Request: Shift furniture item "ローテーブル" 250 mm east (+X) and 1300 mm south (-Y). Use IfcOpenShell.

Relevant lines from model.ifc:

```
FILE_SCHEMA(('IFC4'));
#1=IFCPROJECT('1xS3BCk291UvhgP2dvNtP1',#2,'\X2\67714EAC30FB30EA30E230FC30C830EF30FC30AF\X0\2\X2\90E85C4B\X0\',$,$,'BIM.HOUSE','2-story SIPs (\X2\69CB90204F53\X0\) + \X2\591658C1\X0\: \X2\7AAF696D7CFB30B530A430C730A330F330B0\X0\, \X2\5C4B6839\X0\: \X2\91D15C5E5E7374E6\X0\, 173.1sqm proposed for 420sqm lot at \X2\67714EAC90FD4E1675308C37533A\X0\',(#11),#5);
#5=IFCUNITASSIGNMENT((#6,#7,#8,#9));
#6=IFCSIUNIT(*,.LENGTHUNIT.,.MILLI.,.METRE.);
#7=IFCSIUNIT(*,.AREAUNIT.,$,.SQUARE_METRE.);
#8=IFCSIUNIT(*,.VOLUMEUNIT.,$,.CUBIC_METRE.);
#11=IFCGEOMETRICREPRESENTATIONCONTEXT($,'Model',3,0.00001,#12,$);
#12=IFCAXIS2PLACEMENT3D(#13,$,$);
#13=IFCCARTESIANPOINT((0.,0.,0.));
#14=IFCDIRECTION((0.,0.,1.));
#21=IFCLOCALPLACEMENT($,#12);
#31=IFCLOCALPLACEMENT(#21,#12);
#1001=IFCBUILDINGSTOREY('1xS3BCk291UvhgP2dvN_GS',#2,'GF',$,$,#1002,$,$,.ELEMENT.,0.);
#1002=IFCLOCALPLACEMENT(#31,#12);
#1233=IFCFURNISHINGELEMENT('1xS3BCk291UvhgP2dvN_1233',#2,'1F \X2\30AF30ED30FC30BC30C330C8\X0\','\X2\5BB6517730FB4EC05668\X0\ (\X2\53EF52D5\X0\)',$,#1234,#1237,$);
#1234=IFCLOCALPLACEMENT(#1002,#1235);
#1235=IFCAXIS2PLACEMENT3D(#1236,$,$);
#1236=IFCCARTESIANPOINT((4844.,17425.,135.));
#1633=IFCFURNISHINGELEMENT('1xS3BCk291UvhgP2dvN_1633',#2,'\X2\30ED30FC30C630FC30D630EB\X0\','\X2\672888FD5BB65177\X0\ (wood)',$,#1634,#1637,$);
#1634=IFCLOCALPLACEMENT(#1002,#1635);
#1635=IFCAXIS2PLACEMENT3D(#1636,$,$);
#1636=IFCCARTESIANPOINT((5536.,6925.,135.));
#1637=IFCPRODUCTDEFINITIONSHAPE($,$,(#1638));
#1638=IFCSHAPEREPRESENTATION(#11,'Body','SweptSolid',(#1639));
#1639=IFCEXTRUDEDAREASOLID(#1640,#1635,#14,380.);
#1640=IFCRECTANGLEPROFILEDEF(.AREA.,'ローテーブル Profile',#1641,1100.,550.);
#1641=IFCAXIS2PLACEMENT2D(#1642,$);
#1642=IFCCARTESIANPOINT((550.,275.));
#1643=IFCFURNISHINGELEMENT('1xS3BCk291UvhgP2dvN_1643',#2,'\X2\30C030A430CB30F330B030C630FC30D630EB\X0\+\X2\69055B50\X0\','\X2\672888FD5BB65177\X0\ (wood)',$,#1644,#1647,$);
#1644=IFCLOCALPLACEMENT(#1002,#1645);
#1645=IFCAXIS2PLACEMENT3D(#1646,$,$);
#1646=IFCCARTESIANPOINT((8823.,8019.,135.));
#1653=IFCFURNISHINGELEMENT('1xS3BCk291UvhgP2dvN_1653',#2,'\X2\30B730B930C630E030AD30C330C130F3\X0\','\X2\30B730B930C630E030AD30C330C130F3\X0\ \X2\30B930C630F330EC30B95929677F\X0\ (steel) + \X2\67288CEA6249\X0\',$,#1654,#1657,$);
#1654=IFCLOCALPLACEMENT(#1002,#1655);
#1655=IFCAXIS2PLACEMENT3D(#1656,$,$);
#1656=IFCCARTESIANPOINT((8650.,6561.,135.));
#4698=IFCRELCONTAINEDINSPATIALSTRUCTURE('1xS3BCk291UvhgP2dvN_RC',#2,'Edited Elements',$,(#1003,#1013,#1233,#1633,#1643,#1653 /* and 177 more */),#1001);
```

```python
import ifcopenshell
import ifcopenshell.api.geometry
import ifcopenshell.util.placement
import ifcopenshell.util.unit

model = ifcopenshell.open("model.ifc")
unit_scale = ifcopenshell.util.unit.calculate_unit_scale(model)

item = model.by_guid("1xS3BCk291UvhgP2dvN_1633")
matrix = ifcopenshell.util.placement.get_local_placement(item.ObjectPlacement)
matrix[0, 3] += 0.25 / unit_scale
matrix[1, 3] -= 1.3 / unit_scale
ifcopenshell.api.geometry.edit_object_placement(model, product=item, matrix=matrix, is_si=False)

print(ifcopenshell.util.placement.get_local_placement(item.ObjectPlacement).round(3) + 0.0)

model.write("model_rev.ifc")
```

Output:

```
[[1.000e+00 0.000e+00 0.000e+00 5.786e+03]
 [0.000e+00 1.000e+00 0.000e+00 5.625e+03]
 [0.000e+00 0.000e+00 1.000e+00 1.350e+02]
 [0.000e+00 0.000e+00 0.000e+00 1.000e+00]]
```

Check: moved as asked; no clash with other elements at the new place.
